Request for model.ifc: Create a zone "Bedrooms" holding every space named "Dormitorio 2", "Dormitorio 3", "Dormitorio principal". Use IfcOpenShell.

First a look at what the model holds.

```python
import ifcopenshell

model = ifcopenshell.open("model.ifc")
print(model.schema)
seen = {}
for space in model.by_type("IfcSpace"):
    seen[space.LongName] = seen.get(space.LongName, 0) + 1
for name, count in sorted(seen.items(), key=str):
    print(count, "x", name)
print("zones:", [z.Name for z in model.by_type("IfcZone")][:20])
```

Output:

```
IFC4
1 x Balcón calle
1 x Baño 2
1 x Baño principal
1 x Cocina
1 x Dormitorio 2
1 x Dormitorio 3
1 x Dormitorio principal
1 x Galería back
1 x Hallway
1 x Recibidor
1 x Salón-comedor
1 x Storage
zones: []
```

```python
import ifcopenshell
import ifcopenshell.api.group
import ifcopenshell.api.root

model = ifcopenshell.open("model.ifc")

names = {"Dormitorio 2", "Dormitorio 3", "Dormitorio principal"}
spaces = [s for s in model.by_type("IfcSpace") if s.LongName in names]

zone = ifcopenshell.api.root.create_entity(model, ifc_class="IfcZone", name="Bedrooms")
ifcopenshell.api.group.assign_group(model, products=spaces, group=zone)
print(len(spaces), "spaces in", zone.Name)

model.write("model_edited.ifc")
```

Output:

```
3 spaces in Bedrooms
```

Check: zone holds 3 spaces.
